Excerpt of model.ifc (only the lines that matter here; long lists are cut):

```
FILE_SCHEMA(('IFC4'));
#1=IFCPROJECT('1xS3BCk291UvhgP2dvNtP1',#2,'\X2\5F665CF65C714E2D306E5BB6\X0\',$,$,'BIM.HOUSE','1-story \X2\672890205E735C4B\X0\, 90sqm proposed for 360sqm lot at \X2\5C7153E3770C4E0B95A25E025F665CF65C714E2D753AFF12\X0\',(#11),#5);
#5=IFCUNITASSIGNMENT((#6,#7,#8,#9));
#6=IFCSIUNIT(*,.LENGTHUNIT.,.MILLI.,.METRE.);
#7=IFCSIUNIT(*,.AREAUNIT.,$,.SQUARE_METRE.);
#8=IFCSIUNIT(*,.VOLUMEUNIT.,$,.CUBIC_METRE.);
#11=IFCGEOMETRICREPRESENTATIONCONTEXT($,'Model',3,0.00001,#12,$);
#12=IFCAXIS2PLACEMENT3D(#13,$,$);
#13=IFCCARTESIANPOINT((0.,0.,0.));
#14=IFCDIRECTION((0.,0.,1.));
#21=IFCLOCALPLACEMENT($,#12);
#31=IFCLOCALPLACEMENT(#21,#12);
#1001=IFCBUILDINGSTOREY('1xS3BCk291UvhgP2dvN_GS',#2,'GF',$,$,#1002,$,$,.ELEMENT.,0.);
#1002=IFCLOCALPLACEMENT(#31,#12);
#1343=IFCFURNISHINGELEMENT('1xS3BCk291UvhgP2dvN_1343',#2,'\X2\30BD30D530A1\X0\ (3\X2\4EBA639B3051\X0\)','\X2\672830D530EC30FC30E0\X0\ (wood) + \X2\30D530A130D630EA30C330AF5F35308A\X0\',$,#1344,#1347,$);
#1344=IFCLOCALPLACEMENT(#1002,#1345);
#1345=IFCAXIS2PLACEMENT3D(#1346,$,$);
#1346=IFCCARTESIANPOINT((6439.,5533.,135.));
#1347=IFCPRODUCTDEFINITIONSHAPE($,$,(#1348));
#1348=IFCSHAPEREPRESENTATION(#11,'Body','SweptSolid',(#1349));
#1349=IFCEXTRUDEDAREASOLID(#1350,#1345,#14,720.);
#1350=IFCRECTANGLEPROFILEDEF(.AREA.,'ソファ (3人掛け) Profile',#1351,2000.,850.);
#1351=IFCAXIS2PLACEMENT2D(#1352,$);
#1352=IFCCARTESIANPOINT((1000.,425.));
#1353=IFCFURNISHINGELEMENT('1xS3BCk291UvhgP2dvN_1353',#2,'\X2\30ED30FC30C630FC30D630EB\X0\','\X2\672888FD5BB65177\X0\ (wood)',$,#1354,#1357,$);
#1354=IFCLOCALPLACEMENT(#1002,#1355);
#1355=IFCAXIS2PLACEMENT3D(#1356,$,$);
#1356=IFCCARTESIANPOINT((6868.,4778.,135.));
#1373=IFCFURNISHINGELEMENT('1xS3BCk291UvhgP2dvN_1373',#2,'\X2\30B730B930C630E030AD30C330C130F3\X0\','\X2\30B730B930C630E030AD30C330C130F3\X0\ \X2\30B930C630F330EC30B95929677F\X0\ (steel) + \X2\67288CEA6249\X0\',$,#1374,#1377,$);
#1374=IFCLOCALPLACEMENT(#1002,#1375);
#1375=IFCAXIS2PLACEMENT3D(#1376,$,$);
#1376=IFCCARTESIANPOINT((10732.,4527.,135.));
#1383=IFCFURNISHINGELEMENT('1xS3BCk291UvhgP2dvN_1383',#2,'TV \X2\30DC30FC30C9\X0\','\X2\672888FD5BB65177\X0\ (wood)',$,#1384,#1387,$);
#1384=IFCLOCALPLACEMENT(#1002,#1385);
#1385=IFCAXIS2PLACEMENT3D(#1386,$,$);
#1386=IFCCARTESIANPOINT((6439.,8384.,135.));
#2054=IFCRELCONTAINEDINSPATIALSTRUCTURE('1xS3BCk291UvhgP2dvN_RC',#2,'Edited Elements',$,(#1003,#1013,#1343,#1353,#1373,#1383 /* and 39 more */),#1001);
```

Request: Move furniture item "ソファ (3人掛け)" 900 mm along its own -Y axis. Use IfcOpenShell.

```python
import ifcopenshell
import ifcopenshell.api.geometry
import ifcopenshell.util.placement

model = ifcopenshell.open("model.ifc")

item = model.by_id(1343)
matrix = ifcopenshell.util.placement.get_local_placement(item.ObjectPlacement)
matrix[:3, 3] -= matrix[:3, 1] * 900.0
ifcopenshell.api.geometry.edit_object_placement(model, product=item, matrix=matrix, is_si=False)

print(ifcopenshell.util.placement.get_local_placement(item.ObjectPlacement).round(3) + 0.0)

model.write("model_edited.ifc")
```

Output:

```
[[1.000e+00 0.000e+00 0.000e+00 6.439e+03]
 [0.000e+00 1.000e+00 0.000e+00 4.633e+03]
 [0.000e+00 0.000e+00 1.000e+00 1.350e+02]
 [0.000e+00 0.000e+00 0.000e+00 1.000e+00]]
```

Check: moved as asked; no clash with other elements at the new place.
